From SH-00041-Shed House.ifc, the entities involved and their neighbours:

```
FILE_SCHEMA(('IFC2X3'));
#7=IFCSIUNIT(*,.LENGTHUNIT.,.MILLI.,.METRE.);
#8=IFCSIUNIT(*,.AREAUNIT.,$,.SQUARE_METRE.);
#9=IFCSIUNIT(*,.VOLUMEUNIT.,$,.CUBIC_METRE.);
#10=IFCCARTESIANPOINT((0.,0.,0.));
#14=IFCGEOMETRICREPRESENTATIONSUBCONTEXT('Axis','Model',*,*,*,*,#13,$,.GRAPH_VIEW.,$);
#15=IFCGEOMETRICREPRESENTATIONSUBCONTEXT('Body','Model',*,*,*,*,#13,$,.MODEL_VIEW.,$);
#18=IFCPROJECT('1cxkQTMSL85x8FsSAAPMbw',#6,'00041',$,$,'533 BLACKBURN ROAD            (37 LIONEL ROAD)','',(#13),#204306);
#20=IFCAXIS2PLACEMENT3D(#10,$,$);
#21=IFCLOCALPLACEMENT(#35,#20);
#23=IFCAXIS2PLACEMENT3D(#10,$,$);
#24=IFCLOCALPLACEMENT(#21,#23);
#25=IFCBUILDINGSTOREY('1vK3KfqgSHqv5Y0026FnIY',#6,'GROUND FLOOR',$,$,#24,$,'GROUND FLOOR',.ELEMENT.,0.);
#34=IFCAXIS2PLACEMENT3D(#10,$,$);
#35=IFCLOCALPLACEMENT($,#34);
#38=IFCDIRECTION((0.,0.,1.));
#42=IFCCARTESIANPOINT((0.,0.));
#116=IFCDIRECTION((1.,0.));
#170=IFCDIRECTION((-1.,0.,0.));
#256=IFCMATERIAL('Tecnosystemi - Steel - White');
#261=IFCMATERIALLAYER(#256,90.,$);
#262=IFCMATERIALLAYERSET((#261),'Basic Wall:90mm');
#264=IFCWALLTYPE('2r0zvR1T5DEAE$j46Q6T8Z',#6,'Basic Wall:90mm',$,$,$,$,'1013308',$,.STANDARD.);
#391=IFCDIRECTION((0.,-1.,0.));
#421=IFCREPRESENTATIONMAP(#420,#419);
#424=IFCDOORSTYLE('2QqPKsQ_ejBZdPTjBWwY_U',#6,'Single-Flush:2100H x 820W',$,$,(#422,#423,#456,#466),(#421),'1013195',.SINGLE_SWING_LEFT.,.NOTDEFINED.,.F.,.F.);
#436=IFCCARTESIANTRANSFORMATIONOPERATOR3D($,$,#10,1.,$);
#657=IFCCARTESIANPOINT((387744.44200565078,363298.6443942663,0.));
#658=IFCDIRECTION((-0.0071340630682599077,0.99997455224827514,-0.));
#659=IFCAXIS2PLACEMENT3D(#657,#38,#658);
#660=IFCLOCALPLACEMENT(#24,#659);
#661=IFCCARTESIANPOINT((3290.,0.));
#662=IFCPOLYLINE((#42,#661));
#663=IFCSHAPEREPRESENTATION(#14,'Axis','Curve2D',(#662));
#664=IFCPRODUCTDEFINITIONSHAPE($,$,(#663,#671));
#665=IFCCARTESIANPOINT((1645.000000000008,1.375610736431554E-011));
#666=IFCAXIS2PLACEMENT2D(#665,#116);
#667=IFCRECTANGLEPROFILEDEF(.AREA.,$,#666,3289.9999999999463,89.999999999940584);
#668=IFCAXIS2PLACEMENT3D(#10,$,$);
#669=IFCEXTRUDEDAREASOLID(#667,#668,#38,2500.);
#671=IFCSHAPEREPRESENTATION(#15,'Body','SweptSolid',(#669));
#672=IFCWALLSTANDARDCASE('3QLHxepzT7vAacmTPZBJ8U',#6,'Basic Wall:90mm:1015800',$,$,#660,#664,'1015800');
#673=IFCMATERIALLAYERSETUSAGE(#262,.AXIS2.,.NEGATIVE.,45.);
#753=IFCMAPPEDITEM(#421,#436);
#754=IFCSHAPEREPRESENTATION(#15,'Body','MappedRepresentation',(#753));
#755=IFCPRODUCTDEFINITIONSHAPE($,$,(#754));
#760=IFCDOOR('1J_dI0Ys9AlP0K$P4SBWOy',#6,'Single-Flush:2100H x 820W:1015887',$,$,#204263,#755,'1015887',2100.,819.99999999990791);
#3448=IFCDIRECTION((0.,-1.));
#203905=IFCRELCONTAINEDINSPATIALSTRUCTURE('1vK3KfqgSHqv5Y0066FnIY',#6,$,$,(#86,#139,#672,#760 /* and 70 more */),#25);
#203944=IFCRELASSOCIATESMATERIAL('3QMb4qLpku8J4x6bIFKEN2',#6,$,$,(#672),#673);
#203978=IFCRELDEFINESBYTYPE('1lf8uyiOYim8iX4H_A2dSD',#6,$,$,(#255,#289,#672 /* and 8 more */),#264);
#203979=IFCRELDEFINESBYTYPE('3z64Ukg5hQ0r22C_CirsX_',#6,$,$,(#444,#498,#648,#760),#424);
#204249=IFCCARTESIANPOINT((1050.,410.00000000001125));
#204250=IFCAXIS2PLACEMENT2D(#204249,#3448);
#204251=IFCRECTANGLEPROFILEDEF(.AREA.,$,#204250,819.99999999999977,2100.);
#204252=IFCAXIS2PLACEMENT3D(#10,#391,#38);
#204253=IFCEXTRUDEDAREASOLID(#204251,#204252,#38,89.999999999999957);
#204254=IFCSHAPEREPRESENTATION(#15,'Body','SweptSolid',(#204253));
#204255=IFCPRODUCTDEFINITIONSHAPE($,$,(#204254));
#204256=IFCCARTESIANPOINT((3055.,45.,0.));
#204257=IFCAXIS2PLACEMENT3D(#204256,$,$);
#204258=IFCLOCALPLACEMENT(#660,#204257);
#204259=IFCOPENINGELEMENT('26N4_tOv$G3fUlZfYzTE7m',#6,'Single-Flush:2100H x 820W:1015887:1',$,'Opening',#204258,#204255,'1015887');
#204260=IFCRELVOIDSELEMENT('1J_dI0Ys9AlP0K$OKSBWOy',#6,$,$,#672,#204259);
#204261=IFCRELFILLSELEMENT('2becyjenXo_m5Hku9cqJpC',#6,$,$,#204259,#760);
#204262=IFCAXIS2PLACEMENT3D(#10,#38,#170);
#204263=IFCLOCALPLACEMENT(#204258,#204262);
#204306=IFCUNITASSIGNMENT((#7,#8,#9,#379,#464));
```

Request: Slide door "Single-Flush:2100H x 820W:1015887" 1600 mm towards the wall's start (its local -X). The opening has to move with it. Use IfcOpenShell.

```python
import ifcopenshell
import ifcopenshell.api.geometry
import ifcopenshell.util.placement

model = ifcopenshell.open("SH-00041-Shed House.ifc")

door = model.by_id(760)
opening = door.FillsVoids[0].RelatingOpeningElement
wall = opening.VoidsElements[0].RelatingBuildingElement

wall_matrix = ifcopenshell.util.placement.get_local_placement(wall.ObjectPlacement)
shift = wall_matrix[:3, 0] * -1600.0
before = ifcopenshell.util.placement.get_local_placement(door.ObjectPlacement)[:3, 3].copy()

# The door is placed relative to its opening, so it follows when the opening moves.
matrix = ifcopenshell.util.placement.get_local_placement(opening.ObjectPlacement)
matrix[:3, 3] += shift
ifcopenshell.api.geometry.edit_object_placement(
    model, product=opening, matrix=matrix, is_si=False, should_transform_children=True
)

after = ifcopenshell.util.placement.get_local_placement(door.ObjectPlacement)[:3, 3]
print("door moved by", (after - before).round(3) + 0.0)

model.write("SH-00041-Shed House-out.ifc")
```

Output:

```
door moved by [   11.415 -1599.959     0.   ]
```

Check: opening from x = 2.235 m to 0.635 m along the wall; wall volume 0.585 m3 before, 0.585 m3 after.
